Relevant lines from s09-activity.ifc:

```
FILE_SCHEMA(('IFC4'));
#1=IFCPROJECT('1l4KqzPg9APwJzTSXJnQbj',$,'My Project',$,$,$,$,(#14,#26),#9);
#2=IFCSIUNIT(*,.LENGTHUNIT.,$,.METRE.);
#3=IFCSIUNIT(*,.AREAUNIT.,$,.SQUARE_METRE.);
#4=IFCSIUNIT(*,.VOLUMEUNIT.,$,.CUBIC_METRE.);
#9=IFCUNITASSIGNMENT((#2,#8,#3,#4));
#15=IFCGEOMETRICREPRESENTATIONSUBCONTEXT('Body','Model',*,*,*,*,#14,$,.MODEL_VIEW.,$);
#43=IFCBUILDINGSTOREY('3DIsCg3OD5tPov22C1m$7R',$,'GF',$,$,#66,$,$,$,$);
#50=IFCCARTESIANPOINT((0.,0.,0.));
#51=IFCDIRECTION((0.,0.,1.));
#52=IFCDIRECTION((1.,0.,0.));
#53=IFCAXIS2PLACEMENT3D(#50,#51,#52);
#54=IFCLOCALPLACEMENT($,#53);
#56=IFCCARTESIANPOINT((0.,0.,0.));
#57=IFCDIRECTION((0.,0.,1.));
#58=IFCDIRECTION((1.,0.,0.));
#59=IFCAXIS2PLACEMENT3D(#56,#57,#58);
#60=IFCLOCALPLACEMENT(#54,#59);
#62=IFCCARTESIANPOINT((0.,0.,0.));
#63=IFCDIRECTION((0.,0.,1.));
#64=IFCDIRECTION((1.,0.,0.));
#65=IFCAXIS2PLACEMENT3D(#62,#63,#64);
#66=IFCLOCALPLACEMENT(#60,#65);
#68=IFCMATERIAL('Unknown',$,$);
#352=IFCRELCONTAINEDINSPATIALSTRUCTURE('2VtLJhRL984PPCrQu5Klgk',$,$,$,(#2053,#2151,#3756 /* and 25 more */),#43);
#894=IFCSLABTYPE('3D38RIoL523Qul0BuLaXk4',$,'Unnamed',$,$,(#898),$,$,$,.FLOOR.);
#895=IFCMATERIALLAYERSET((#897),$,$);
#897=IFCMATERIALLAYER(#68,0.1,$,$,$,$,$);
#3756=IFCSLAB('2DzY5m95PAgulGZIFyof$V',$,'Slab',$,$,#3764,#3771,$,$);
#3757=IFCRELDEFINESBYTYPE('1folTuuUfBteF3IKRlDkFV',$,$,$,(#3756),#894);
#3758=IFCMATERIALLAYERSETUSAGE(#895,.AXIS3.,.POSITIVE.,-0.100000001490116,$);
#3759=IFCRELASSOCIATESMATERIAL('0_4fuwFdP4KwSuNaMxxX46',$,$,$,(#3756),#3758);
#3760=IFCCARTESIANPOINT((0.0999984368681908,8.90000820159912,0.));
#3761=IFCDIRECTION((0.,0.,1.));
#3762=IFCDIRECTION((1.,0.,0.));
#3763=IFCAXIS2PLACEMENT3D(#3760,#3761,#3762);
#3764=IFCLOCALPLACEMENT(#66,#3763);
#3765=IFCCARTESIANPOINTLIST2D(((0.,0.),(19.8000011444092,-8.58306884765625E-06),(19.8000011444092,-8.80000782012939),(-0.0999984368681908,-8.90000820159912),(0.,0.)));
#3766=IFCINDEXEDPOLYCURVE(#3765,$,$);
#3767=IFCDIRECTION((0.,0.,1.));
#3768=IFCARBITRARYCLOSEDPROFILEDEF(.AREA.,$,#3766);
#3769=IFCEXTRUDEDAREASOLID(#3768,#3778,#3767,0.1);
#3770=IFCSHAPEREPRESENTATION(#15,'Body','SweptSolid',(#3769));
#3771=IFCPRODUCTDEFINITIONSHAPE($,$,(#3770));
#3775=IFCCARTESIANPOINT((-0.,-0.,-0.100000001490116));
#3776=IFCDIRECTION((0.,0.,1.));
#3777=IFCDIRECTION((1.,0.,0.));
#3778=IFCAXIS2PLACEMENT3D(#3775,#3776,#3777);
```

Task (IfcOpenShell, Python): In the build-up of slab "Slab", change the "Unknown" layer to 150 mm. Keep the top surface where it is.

```python
import ifcopenshell
import ifcopenshell.util.element
import ifcopenshell.util.representation

model = ifcopenshell.open("s09-activity.ifc")

layer_set = model.by_id(895)
layer = next(l for l in layer_set.MaterialLayers if l.Material and l.Material.Name == "Unknown")
change = 0.15 - layer.LayerThickness
layer.LayerThickness += change

# Geometry does not follow the layer set by itself.
slabs = [e for e in ifcopenshell.util.element.get_elements_by_material(model, layer_set) if e.is_a("IfcSlab")]
for slab in sorted(slabs, key=lambda e: e.id()):
    body = ifcopenshell.util.representation.get_representation(slab, "Model", "Body")
    solid = body.Items[0]
    old_depth = solid.Depth
    solid.Depth += change
    # Extruded upwards: lower the start of the extrusion so the top stays.
    x, y, z = solid.Position.Location.Coordinates
    solid.Position.Location = model.createIfcCartesianPoint((x, y, z - change))
    print(slab.id(), f"{old_depth:g} -> {solid.Depth:g}")

# The layers are counted up from the underside, which has moved.
for usage in {ifcopenshell.util.element.get_material(slab) for slab in slabs}:
    usage.OffsetFromReferenceLine -= change

model.write("s09-activity_v2.ifc")
```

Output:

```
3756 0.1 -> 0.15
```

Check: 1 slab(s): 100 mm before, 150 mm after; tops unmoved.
